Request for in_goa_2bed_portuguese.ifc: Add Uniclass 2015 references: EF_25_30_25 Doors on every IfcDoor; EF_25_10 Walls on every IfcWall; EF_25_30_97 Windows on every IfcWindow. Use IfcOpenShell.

First a look at what the model holds.

```python
import ifcopenshell

model = ifcopenshell.open("in_goa_2bed_portuguese.ifc")
print(model.schema)
print("classifications:", [c.Name for c in model.by_type("IfcClassification")])
for ifc_class in ("IfcDoor", "IfcRoof", "IfcStair", "IfcWall", "IfcWindow"):
    print(ifc_class, len(model.by_type(ifc_class)))
```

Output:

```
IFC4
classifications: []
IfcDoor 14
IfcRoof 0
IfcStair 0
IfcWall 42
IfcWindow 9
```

```python
import ifcopenshell
import ifcopenshell.api.classification

model = ifcopenshell.open("in_goa_2bed_portuguese.ifc")

system = ifcopenshell.api.classification.add_classification(model, classification="Uniclass 2015")

codes = {
    "IfcDoor": ("EF_25_30_25", "Doors"),
    "IfcWall": ("EF_25_10", "Walls"),
    "IfcWindow": ("EF_25_30_97", "Windows"),
}
for ifc_class, (code, name) in codes.items():
    products = model.by_type(ifc_class)
    ifcopenshell.api.classification.add_reference(
        model, products=products, classification=system, identification=code, name=name
    )
    print(code, len(products))

model.write("in_goa_2bed_portuguese-out.ifc")
```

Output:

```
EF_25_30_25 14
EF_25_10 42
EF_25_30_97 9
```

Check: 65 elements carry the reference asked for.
